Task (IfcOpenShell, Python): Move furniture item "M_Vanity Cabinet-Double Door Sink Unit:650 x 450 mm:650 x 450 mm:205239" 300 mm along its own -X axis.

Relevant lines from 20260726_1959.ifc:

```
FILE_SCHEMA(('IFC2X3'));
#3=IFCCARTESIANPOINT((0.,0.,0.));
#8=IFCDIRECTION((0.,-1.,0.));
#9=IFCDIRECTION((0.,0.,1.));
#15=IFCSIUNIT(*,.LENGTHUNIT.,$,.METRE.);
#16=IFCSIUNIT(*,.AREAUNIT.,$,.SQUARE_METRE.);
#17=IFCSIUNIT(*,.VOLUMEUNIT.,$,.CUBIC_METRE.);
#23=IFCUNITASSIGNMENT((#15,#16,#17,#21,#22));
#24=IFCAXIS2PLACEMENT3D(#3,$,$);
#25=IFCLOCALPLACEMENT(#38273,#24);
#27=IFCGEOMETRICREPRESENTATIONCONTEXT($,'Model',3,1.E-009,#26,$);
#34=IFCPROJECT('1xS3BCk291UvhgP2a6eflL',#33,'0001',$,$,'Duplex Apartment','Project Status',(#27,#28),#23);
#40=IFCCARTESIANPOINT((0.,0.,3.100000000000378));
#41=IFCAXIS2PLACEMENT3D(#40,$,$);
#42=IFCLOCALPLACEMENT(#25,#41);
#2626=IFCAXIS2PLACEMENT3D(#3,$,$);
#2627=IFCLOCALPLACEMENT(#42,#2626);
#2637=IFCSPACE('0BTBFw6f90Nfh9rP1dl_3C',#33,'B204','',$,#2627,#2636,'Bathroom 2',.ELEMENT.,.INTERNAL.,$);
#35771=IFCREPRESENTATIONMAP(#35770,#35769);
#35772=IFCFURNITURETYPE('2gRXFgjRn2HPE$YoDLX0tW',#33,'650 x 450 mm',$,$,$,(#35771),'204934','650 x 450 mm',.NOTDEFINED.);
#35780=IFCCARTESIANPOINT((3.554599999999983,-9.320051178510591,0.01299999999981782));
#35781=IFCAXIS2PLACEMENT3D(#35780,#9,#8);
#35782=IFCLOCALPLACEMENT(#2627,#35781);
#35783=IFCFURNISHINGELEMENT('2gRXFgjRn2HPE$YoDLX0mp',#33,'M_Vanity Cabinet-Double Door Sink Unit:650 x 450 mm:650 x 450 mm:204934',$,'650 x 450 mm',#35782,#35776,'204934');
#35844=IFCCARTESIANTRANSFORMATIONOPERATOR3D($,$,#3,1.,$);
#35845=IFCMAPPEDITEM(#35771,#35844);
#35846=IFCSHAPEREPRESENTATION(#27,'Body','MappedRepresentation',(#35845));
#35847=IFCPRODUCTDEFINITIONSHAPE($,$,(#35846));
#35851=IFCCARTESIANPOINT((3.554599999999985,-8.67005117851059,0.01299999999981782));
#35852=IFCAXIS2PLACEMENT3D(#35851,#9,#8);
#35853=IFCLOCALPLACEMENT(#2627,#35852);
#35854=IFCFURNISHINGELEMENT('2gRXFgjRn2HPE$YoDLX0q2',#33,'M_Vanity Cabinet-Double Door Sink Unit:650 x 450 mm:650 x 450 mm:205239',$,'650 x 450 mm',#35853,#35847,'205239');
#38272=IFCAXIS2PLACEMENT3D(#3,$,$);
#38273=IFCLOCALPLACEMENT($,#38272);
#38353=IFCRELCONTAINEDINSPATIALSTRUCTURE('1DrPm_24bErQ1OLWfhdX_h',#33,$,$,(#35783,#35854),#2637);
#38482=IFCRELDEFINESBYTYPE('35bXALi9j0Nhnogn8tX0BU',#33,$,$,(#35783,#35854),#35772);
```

```python
import ifcopenshell
import ifcopenshell.api.geometry
import ifcopenshell.util.placement
import ifcopenshell.util.unit

model = ifcopenshell.open("20260726_1959.ifc")
unit_scale = ifcopenshell.util.unit.calculate_unit_scale(model)

item = model.by_guid("2gRXFgjRn2HPE$YoDLX0q2")
matrix = ifcopenshell.util.placement.get_local_placement(item.ObjectPlacement)
matrix[:3, 3] -= matrix[:3, 0] * 0.3 / unit_scale
ifcopenshell.api.geometry.edit_object_placement(model, product=item, matrix=matrix, is_si=False)

print(ifcopenshell.util.placement.get_local_placement(item.ObjectPlacement).round(3) + 0.0)

model.write("20260726_1959_updated.ifc")
```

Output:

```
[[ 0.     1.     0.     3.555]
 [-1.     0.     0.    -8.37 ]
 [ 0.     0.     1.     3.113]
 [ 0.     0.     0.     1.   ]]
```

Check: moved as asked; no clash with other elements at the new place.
